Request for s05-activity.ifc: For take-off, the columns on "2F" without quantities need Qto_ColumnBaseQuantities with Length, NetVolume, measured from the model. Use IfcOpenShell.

First a look at what the model holds.

```python
import ifcopenshell
import ifcopenshell.util.element
import ifcopenshell.util.unit

model = ifcopenshell.open("s05-activity.ifc")
print(model.schema)
for unit_type in ("LENGTHUNIT", "AREAUNIT", "VOLUMEUNIT"):
    print(unit_type, ifcopenshell.util.unit.calculate_unit_scale(model, unit_type))
storey = next(s for s in model.by_type("IfcBuildingStorey") if s.Name == "2F")
columns = [e for e in ifcopenshell.util.element.get_decomposition(storey) if e.is_a("IfcColumn")]
for e in sorted(columns, key=lambda e: e.id()):
    print(e.id(), e.is_a(), e.Name, list(ifcopenshell.util.element.get_psets(e, qtos_only=True)), sep=" | ")
```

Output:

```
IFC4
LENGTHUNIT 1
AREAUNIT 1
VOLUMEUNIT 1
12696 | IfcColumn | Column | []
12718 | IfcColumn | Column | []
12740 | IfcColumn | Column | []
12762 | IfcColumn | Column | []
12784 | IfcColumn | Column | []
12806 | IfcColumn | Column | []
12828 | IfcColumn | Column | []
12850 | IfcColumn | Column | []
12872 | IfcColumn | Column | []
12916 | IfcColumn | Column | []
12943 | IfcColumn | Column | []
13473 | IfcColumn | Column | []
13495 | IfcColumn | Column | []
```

```python
import ifcopenshell
import ifcopenshell.api.pset
import ifcopenshell.geom
import ifcopenshell.util.element
import ifcopenshell.util.shape
import ifcopenshell.util.unit

model = ifcopenshell.open("s05-activity.ifc")
unit_scale = ifcopenshell.util.unit.calculate_unit_scale(model)
volume_scale = ifcopenshell.util.unit.calculate_unit_scale(model, "VOLUMEUNIT")
settings = ifcopenshell.geom.settings()

storey = next(s for s in model.by_type("IfcBuildingStorey") if s.Name == "2F")
columns = [e for e in ifcopenshell.util.element.get_decomposition(storey) if e.is_a("IfcColumn")]

for e in sorted(columns, key=lambda e: e.id()):
    if ifcopenshell.util.element.get_psets(e, qtos_only=True, should_inherit=False):
        continue
    # Geometry comes back in metres, in the element's own axes.
    shape = ifcopenshell.geom.create_shape(settings, e)
    values = {
        "Length": ifcopenshell.util.shape.get_z(shape.geometry) / unit_scale,
        "NetVolume": ifcopenshell.util.shape.get_volume(shape.geometry) / volume_scale,
    }
    qto = ifcopenshell.api.pset.add_qto(model, product=e, name="Qto_ColumnBaseQuantities")
    ifcopenshell.api.pset.edit_qto(model, qto=qto, properties=values)
    print(e.id(), {k: round(v, 3) for k, v in values.items()})

model.write("s05-activity_v2.ifc")
```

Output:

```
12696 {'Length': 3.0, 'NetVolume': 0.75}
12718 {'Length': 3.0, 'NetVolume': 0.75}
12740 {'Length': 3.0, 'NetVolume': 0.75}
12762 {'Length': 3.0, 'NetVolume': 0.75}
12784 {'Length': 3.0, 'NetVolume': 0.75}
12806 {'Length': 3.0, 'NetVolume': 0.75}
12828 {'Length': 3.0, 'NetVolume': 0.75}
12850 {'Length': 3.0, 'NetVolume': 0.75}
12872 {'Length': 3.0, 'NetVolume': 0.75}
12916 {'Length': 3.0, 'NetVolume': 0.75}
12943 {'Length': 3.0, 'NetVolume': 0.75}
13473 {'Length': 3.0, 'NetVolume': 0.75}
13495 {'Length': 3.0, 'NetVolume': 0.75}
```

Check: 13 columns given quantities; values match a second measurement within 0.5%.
